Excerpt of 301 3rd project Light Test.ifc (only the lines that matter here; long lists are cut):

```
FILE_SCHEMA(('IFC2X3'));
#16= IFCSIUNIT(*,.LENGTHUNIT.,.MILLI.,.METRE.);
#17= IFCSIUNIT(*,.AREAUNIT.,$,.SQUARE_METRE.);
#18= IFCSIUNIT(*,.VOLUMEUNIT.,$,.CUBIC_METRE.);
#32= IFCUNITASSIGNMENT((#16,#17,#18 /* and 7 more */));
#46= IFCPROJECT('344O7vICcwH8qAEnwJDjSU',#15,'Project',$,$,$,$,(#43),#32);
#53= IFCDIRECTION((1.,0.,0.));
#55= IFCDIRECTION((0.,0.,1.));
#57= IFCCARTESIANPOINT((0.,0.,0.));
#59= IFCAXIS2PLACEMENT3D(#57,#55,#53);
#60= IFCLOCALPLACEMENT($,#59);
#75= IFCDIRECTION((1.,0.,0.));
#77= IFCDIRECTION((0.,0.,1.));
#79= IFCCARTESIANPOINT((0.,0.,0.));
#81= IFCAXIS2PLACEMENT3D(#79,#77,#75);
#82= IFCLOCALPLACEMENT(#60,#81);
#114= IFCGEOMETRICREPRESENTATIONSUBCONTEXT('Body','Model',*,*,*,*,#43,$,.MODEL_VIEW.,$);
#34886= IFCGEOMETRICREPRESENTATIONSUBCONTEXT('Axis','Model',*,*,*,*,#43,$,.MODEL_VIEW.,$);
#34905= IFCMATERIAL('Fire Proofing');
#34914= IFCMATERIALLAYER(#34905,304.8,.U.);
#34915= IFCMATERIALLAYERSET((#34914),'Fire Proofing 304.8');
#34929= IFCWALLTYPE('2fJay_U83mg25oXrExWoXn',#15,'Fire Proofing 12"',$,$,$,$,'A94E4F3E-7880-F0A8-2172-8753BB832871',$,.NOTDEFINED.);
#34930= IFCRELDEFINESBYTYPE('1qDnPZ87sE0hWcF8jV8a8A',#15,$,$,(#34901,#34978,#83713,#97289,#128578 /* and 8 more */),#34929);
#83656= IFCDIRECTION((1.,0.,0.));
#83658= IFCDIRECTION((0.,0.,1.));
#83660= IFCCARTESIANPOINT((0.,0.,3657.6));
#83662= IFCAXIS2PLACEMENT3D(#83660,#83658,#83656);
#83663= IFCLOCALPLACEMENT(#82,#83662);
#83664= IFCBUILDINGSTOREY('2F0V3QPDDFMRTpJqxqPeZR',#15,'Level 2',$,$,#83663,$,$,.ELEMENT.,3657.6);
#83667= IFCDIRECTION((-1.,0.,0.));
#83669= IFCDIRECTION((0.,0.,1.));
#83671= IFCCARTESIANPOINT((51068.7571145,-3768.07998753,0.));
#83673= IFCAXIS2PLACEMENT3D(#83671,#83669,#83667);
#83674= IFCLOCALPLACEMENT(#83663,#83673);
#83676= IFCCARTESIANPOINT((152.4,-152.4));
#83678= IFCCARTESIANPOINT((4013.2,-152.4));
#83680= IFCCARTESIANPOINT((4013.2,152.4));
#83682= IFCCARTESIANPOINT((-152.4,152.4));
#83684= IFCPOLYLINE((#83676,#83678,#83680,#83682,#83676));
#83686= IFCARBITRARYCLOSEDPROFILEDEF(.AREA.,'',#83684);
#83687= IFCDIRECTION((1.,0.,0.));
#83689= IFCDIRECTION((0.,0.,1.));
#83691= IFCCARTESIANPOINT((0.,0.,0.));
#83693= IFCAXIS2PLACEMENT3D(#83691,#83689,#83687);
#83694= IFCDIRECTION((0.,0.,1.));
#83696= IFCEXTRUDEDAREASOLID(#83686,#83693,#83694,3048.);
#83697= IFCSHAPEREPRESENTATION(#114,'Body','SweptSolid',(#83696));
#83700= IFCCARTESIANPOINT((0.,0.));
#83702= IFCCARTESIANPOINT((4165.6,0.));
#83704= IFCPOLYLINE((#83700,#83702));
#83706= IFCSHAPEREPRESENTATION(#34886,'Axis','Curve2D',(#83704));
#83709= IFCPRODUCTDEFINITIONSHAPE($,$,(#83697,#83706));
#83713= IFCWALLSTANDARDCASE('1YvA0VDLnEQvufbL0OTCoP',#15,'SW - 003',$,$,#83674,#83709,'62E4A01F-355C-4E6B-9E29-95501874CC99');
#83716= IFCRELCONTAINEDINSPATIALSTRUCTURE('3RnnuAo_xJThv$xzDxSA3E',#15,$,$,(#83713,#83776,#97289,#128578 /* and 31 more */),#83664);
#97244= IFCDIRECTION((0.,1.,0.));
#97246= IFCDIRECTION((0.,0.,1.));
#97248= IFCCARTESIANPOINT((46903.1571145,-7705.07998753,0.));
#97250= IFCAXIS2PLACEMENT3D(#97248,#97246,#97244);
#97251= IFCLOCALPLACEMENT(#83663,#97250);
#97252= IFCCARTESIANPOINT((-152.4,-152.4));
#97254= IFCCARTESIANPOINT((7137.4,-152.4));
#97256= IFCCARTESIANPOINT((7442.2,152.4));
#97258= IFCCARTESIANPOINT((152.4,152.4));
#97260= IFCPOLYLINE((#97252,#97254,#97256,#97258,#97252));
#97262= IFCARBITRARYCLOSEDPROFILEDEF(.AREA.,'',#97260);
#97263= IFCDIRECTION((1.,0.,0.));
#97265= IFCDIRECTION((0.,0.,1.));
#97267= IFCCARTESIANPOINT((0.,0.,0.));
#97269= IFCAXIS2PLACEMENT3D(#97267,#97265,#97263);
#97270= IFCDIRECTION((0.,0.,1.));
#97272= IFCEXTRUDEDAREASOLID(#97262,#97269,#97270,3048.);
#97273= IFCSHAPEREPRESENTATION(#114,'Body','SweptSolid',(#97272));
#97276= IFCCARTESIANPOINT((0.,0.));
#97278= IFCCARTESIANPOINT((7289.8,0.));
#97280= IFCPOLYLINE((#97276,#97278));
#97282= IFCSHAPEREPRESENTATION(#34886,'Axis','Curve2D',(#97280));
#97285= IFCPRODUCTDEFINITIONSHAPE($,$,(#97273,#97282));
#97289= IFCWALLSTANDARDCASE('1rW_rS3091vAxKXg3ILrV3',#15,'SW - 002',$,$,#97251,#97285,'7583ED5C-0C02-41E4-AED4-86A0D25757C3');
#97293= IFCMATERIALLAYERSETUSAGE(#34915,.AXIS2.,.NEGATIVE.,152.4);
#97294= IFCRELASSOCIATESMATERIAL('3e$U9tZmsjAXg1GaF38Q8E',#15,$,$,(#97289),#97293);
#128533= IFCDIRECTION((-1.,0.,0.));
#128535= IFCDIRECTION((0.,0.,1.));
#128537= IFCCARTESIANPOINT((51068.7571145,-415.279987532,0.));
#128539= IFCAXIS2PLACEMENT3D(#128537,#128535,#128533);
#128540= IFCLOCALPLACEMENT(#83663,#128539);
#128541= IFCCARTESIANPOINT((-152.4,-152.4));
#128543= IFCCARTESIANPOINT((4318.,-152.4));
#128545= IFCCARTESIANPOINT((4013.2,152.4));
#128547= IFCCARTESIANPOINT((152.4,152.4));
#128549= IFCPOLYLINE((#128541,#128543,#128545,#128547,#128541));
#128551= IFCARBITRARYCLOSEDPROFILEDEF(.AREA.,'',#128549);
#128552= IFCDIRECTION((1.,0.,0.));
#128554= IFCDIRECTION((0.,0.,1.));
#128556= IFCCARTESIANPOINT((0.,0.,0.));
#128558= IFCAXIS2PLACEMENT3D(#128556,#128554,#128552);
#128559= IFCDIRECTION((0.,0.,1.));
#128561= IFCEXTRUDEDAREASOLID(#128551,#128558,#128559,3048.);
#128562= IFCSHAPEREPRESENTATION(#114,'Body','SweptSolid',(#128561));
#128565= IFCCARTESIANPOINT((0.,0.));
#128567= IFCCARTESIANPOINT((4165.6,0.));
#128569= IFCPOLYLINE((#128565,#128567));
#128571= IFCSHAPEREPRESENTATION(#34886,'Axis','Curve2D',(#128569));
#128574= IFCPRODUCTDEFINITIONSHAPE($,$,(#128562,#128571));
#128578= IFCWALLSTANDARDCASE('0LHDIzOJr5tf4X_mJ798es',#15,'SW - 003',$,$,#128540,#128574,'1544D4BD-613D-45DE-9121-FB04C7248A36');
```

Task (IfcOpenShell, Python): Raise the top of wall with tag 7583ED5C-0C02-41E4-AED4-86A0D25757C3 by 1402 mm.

```python
import ifcopenshell
import ifcopenshell.geom
import ifcopenshell.util.representation
import ifcopenshell.util.shape

model = ifcopenshell.open("301 3rd project Light Test.ifc")
settings = ifcopenshell.geom.settings()


def volume(element):
    """Net volume in cubic metres, openings subtracted."""
    shape = ifcopenshell.geom.create_shape(settings, element)
    return ifcopenshell.util.shape.get_volume(shape.geometry)


wall = model.by_id(97289)
before = volume(wall)

body = ifcopenshell.util.representation.get_representation(wall, "Model", "Body")
solid = body.Items[0]
old_height = solid.Depth
solid.Depth += 1402.0
after = volume(wall)

print(f"height {old_height:g} -> {solid.Depth:g}, volume {before:.3f} -> {after:.3f} m3")

model.write("301 3rd project Light Test_rev.ifc")
```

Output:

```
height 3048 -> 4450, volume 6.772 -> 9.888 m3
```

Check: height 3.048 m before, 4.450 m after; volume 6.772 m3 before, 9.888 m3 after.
